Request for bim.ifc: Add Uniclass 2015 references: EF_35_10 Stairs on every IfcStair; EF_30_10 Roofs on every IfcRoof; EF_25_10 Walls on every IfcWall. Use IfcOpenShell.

First a look at what the model holds.

```python
import ifcopenshell

model = ifcopenshell.open("bim.ifc")
print(model.schema)
print("classifications:", [c.Name for c in model.by_type("IfcClassification")])
for ifc_class in ("IfcDoor", "IfcRoof", "IfcStair", "IfcWall", "IfcWindow"):
    print(ifc_class, len(model.by_type(ifc_class)))
```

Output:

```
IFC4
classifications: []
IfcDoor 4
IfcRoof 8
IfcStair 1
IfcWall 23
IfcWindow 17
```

```python
import ifcopenshell
import ifcopenshell.api.classification

model = ifcopenshell.open("bim.ifc")

system = ifcopenshell.api.classification.add_classification(model, classification="Uniclass 2015")

codes = {
    "IfcStair": ("EF_35_10", "Stairs"),
    "IfcRoof": ("EF_30_10", "Roofs"),
    "IfcWall": ("EF_25_10", "Walls"),
}
for ifc_class, (code, name) in codes.items():
    products = model.by_type(ifc_class)
    ifcopenshell.api.classification.add_reference(
        model, products=products, classification=system, identification=code, name=name
    )
    print(code, len(products))

model.write("bim_rev.ifc")
```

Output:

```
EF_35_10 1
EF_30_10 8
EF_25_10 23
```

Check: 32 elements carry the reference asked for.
